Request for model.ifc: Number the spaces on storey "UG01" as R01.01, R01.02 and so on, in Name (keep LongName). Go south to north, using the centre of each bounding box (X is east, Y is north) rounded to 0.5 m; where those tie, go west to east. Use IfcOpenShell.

First a look at what the model holds.

```python
import ifcopenshell
import ifcopenshell.util.element
import ifcopenshell.util.placement

model = ifcopenshell.open("model.ifc")
print(model.schema)
storey = next(s for s in model.by_type("IfcBuildingStorey") if s.Name == "UG01")
spaces = [e for e in ifcopenshell.util.element.get_decomposition(storey) if e.is_a("IfcSpace")]
for e in sorted(spaces, key=lambda e: e.id()):
    origin = ifcopenshell.util.placement.get_local_placement(e.ObjectPlacement)[:3, 3]
    print(e.id(), e.Name, e.LongName, origin.round(2) + 0.0, sep=" | ")
```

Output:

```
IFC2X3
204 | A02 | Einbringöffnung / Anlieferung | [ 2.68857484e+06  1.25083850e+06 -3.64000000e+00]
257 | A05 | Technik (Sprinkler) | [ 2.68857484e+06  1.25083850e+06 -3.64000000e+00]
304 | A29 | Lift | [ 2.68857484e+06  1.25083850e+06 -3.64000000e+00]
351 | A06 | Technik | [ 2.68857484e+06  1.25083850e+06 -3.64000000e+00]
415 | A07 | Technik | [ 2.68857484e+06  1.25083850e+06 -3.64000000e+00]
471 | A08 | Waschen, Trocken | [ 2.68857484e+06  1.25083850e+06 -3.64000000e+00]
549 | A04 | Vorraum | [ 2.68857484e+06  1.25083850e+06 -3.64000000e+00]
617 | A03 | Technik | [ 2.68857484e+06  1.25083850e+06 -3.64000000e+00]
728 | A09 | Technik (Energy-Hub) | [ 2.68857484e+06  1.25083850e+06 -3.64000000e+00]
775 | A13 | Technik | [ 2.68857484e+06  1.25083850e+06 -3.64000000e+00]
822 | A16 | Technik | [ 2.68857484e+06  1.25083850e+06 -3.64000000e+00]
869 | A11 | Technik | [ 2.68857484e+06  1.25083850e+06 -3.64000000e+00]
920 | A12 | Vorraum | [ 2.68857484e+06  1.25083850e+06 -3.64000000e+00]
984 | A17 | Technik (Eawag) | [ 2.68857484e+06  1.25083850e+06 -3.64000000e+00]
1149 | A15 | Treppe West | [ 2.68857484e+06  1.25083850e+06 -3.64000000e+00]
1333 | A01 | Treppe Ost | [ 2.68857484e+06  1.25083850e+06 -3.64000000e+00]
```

```python
import ifcopenshell
import ifcopenshell.geom
import ifcopenshell.util.element
import ifcopenshell.util.shape

model = ifcopenshell.open("model.ifc")
settings = ifcopenshell.geom.settings()
settings.set("use-world-coords", True)


def centre(element):
    shape = ifcopenshell.geom.create_shape(settings, element)
    return ifcopenshell.util.shape.get_bbox_centroid(shape.geometry)


storey = next(s for s in model.by_type("IfcBuildingStorey") if s.Name == "UG01")
spaces = [e for e in ifcopenshell.util.element.get_decomposition(storey) if e.is_a("IfcSpace")]

# Insertion points can sit at a corner or the storey origin, so sort by the geometry (in metres).
centres = {e: centre(e) for e in spaces}
spaces.sort(key=lambda e: (round(centres[e][1] / 0.5), centres[e][0]))

for i, e in enumerate(spaces, start=1):
    number = f"R01.{i:02d}"
    e.Name = number
    print(e.id(), number)

model.write("model-out.ifc")
```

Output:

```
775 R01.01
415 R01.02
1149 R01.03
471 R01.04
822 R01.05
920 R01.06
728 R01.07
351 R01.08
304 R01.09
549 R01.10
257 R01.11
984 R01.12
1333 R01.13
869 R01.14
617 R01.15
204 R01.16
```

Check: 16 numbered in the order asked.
